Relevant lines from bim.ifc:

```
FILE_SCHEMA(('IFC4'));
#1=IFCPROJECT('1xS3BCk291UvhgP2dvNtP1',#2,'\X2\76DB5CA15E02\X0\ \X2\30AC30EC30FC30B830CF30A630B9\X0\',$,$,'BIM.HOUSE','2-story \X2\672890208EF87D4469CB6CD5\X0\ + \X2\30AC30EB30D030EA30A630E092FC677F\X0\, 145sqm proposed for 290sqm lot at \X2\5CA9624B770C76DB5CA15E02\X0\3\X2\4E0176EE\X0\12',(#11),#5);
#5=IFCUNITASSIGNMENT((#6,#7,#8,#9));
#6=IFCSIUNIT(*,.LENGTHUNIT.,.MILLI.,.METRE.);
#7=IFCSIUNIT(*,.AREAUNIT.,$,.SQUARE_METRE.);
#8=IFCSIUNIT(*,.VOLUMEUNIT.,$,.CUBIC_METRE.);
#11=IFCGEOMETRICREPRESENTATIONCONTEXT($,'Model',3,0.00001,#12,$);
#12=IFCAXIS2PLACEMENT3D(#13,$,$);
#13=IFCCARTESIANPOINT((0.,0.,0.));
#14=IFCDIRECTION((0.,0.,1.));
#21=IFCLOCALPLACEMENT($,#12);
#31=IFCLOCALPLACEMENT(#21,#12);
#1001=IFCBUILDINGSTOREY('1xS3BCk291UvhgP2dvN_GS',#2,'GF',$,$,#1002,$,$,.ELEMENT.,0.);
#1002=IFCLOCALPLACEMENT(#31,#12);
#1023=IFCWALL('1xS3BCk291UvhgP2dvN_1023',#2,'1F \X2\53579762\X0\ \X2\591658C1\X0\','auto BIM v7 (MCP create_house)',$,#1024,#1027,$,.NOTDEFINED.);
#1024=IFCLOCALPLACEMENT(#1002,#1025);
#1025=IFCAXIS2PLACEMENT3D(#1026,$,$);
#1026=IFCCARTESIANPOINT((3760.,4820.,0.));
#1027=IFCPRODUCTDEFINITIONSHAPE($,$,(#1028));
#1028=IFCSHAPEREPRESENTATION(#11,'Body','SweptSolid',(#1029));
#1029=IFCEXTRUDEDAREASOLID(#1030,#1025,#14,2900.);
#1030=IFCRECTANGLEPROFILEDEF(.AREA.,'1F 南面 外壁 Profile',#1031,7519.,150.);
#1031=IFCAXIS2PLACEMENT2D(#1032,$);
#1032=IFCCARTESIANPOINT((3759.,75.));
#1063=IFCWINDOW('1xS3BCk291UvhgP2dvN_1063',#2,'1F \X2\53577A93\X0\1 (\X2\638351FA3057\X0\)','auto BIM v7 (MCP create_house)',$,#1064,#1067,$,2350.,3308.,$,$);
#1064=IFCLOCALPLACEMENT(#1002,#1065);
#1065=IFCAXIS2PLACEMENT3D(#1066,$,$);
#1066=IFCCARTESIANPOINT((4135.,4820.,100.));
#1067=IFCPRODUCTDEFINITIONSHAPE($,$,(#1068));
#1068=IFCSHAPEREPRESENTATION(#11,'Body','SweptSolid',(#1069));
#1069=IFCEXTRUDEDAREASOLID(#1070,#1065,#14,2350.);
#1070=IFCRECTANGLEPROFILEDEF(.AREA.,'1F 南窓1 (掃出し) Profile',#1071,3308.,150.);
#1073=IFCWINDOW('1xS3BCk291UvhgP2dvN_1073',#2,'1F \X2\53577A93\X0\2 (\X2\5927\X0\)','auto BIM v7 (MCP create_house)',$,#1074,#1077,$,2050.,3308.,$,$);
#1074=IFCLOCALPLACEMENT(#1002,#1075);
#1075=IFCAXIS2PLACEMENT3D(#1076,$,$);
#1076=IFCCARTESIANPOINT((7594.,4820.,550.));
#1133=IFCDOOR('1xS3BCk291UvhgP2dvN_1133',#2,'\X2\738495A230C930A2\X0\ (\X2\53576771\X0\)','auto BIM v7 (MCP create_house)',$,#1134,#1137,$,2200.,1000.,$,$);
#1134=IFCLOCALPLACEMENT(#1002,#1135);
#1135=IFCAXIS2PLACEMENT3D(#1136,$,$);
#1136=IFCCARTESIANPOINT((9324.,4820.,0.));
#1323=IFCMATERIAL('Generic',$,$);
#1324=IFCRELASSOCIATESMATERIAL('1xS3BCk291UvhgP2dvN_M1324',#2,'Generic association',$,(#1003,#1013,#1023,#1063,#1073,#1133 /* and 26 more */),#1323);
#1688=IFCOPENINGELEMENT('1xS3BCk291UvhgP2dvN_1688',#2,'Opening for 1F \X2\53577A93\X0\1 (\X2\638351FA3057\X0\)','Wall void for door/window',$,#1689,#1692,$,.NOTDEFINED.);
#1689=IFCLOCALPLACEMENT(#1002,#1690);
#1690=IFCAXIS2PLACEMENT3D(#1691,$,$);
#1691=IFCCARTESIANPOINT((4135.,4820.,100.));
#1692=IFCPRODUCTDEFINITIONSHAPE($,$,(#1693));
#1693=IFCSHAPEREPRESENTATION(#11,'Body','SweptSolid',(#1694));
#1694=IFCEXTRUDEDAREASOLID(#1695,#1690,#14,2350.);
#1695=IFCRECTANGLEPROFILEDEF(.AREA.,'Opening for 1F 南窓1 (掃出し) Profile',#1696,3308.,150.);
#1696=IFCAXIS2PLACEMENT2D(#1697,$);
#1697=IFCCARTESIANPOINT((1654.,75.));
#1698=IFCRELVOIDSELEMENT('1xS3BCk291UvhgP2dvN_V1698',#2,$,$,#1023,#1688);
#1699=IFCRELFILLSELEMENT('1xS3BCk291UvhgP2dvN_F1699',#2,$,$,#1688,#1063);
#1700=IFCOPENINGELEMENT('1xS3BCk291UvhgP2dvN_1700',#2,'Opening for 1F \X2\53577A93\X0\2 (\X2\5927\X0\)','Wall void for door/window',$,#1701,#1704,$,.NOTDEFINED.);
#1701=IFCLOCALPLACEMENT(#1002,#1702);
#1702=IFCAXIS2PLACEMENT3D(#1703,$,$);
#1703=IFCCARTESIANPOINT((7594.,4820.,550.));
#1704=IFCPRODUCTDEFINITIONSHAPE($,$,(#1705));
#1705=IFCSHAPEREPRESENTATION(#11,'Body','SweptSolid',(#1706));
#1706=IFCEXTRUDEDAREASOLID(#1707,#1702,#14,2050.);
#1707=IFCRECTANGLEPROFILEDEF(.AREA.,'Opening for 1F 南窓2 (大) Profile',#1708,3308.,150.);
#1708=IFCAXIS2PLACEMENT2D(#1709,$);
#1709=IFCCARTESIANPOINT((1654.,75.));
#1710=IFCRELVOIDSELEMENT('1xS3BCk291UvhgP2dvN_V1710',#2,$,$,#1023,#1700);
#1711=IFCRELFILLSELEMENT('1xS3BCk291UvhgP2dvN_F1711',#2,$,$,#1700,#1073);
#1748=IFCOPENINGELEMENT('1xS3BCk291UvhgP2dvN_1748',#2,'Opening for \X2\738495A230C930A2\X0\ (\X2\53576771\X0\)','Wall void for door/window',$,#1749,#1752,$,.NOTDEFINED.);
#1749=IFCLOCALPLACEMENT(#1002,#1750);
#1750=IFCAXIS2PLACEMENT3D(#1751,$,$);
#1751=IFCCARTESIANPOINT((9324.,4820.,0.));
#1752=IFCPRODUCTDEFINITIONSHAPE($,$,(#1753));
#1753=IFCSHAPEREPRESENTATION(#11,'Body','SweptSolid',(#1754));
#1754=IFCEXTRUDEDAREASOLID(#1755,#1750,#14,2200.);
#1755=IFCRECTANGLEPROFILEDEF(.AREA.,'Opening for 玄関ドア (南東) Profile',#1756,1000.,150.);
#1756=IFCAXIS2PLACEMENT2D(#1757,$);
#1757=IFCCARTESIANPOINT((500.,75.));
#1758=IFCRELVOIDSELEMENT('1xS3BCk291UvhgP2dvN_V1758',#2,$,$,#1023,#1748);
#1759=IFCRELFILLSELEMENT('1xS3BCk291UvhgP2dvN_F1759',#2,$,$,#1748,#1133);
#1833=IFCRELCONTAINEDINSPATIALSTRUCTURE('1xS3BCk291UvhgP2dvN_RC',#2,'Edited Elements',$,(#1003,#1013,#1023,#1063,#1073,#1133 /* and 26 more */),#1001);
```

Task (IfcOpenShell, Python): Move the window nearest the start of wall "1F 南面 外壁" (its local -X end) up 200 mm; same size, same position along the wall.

```python
import numpy as np
import ifcopenshell
import ifcopenshell.api.geometry
import ifcopenshell.util.placement
import ifcopenshell.util.unit

model = ifcopenshell.open("bim.ifc")
unit_scale = ifcopenshell.util.unit.calculate_unit_scale(model)

window = model.by_id(1063)
opening = window.FillsVoids[0].RelatingOpeningElement
dz = 200.0

shift = np.array([0.0, 0.0, dz])
# The window is not placed relative to its opening, so move both.
for product in (opening, window):
    matrix = ifcopenshell.util.placement.get_local_placement(product.ObjectPlacement)
    matrix[:3, 3] += shift
    ifcopenshell.api.geometry.edit_object_placement(model, product=product, matrix=matrix, is_si=False)

print(f"moved by {dz * unit_scale:+.3f} m")

model.write("bim-out.ifc")
```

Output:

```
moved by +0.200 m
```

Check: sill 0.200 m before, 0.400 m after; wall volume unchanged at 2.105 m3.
